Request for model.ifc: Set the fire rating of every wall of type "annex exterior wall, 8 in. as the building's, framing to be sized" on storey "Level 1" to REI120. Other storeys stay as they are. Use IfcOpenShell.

First a look at what the model holds.

```python
import ifcopenshell
import ifcopenshell.util.element

model = ifcopenshell.open("model.ifc")
print(model.schema)
storey = next(s for s in model.by_type("IfcBuildingStorey") if s.Name == "Level 1")
walls = [e for e in ifcopenshell.util.element.get_decomposition(storey) if e.is_a("IfcWall")]
seen = {}
for e in walls:
    element_type = ifcopenshell.util.element.get_type(e)
    key = (element_type.Name if element_type != e and element_type else None, ifcopenshell.util.element.get_pset(e, "Pset_WallCommon", "FireRating"))
    seen[key] = seen.get(key, 0) + 1
for (name, value), count in sorted(seen.items(), key=str):
    print(count, "x", name, "|", value)
```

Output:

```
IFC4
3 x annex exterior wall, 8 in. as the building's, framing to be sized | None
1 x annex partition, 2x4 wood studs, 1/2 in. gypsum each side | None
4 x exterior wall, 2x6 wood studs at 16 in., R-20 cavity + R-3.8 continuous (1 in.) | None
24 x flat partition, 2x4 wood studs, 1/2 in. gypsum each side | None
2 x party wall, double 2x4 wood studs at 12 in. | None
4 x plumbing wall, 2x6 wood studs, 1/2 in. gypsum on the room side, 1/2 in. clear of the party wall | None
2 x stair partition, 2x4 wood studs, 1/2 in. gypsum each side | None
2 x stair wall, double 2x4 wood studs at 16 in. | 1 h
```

```python
import ifcopenshell
import ifcopenshell.api.pset
import ifcopenshell.util.element

model = ifcopenshell.open("model.ifc")

storey = next(s for s in model.by_type("IfcBuildingStorey") if s.Name == "Level 1")
walls = [e for e in ifcopenshell.util.element.get_decomposition(storey) if e.is_a("IfcWall")]

count = 0
for e in walls:
    element_type = ifcopenshell.util.element.get_type(e)
    if element_type in (None, e) or element_type.Name != "annex exterior wall, 8 in. as the building's, framing to be sized":
        continue
    # add_pset returns the element's existing set when there is one.
    pset = ifcopenshell.api.pset.add_pset(model, product=e, name="Pset_WallCommon")
    ifcopenshell.api.pset.edit_pset(model, pset=pset, properties={"FireRating": "REI120"})
    count += 1

print(count, "walls updated")

model.write("model_v2.ifc")
```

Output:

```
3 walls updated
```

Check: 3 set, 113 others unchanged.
